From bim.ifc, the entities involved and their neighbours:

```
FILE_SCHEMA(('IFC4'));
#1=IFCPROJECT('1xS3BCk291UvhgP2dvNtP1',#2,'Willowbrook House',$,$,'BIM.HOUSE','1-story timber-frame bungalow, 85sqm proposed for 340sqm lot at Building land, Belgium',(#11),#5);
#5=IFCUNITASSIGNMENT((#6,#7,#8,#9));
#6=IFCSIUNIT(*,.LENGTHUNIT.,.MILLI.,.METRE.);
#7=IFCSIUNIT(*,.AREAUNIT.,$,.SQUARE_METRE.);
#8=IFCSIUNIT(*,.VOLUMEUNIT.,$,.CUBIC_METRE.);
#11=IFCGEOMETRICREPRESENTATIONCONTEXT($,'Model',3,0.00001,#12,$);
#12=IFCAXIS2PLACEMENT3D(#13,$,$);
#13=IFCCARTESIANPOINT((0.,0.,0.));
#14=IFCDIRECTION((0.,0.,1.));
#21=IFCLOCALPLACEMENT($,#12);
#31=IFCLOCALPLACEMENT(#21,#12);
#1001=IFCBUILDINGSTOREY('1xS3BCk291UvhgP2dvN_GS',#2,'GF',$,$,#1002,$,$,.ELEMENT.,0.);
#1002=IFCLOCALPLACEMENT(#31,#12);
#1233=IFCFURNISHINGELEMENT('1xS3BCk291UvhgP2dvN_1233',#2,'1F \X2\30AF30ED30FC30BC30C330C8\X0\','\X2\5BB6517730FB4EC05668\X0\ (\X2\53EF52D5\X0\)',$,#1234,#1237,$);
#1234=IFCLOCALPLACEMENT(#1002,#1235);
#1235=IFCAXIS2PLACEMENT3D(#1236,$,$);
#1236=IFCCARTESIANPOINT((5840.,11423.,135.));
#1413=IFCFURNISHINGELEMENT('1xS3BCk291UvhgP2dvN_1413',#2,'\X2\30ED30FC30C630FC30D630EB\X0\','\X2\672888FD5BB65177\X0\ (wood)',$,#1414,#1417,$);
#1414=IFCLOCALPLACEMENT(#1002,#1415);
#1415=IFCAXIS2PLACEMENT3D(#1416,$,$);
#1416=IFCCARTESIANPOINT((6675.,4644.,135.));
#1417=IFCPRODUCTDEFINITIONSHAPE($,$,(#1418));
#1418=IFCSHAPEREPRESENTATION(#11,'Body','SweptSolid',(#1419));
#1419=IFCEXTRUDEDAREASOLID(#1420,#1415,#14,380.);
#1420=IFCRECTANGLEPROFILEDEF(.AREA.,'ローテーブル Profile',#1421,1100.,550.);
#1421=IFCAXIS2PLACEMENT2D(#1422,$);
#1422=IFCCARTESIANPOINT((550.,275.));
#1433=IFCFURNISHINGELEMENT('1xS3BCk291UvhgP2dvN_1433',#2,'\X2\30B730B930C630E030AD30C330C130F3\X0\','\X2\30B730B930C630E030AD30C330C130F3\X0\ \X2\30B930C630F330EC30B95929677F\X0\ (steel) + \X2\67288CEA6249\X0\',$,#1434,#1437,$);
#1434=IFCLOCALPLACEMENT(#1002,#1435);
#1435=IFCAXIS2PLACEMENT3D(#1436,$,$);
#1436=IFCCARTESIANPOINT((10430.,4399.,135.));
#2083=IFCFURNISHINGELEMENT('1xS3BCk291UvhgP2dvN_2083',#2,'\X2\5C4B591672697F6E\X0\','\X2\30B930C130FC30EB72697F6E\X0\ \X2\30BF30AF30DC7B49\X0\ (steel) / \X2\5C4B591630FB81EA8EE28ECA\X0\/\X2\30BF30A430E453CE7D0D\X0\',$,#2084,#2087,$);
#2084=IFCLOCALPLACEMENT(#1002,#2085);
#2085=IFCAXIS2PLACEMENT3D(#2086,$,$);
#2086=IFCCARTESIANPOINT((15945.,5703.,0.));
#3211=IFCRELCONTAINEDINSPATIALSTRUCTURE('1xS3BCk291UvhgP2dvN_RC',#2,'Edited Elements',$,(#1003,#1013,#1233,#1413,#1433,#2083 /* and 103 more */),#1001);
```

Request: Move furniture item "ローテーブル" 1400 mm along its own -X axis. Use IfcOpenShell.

```python
import ifcopenshell
import ifcopenshell.api.geometry
import ifcopenshell.util.placement

model = ifcopenshell.open("bim.ifc")

item = model.by_id(1413)
matrix = ifcopenshell.util.placement.get_local_placement(item.ObjectPlacement)
matrix[:3, 3] -= matrix[:3, 0] * 1400.0
ifcopenshell.api.geometry.edit_object_placement(model, product=item, matrix=matrix, is_si=False)

print(ifcopenshell.util.placement.get_local_placement(item.ObjectPlacement).round(3) + 0.0)

model.write("bim_edited.ifc")
```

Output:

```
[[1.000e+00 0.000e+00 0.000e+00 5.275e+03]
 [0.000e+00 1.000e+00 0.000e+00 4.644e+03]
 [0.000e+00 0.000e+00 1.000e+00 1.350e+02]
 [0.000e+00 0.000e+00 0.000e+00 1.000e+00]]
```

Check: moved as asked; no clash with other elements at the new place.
